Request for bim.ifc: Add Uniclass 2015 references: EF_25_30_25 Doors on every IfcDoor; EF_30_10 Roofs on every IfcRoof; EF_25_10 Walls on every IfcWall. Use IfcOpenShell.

First a look at what the model holds.

```python
import ifcopenshell

model = ifcopenshell.open("bim.ifc")
print(model.schema)
print("classifications:", [c.Name for c in model.by_type("IfcClassification")])
for ifc_class in ("IfcDoor", "IfcRoof", "IfcStair", "IfcWall", "IfcWindow"):
    print(ifc_class, len(model.by_type(ifc_class)))
```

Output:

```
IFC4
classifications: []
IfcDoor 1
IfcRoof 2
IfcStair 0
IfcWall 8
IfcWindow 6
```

```python
import ifcopenshell
import ifcopenshell.api.classification

model = ifcopenshell.open("bim.ifc")

system = ifcopenshell.api.classification.add_classification(model, classification="Uniclass 2015")

codes = {
    "IfcDoor": ("EF_25_30_25", "Doors"),
    "IfcRoof": ("EF_30_10", "Roofs"),
    "IfcWall": ("EF_25_10", "Walls"),
}
for ifc_class, (code, name) in codes.items():
    products = model.by_type(ifc_class)
    ifcopenshell.api.classification.add_reference(
        model, products=products, classification=system, identification=code, name=name
    )
    print(code, len(products))

model.write("bim_v2.ifc")
```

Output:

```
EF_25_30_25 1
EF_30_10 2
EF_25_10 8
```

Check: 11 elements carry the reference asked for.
